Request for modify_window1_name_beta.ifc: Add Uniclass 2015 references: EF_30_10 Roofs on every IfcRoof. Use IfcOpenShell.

First a look at what the model holds.

```python
import ifcopenshell

model = ifcopenshell.open("modify_window1_name_beta.ifc")
print(model.schema)
print("classifications:", [c.Name for c in model.by_type("IfcClassification")])
for ifc_class in ("IfcDoor", "IfcRoof", "IfcStair", "IfcWall", "IfcWindow"):
    print(ifc_class, len(model.by_type(ifc_class)))
```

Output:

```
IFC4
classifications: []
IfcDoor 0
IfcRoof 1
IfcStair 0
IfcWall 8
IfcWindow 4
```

```python
import ifcopenshell
import ifcopenshell.api.classification

model = ifcopenshell.open("modify_window1_name_beta.ifc")

system = ifcopenshell.api.classification.add_classification(model, classification="Uniclass 2015")

codes = {
    "IfcRoof": ("EF_30_10", "Roofs"),
}
for ifc_class, (code, name) in codes.items():
    products = model.by_type(ifc_class)
    ifcopenshell.api.classification.add_reference(
        model, products=products, classification=system, identification=code, name=name
    )
    print(code, len(products))

model.write("modify_window1_name_beta_updated.ifc")
```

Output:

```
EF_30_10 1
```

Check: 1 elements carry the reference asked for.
